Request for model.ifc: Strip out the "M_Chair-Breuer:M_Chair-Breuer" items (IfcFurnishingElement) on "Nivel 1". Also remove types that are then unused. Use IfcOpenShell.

First a look at what the model holds.

```python
import ifcopenshell
import ifcopenshell.util.element

model = ifcopenshell.open("model.ifc")
print(model.schema)
storey = next(s for s in model.by_type("IfcBuildingStorey") if s.Name == "Nivel 1")
furniture = [e for e in ifcopenshell.util.element.get_decomposition(storey) if e.is_a("IfcFurnishingElement")]
seen = {}
for e in furniture:
    element_type = ifcopenshell.util.element.get_type(e)
    name = element_type.Name if element_type not in (None, e) else None
    seen[name] = seen.get(name, 0) + 1
for name, count in sorted(seen.items(), key=str):
    print(count, "x", name)
```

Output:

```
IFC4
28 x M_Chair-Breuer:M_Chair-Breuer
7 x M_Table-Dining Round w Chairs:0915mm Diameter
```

```python
import ifcopenshell
import ifcopenshell.api.root
import ifcopenshell.util.element

model = ifcopenshell.open("model.ifc")

storey = next(s for s in model.by_type("IfcBuildingStorey") if s.Name == "Nivel 1")
furniture = [e for e in ifcopenshell.util.element.get_decomposition(storey) if e.is_a("IfcFurnishingElement")]
targets = [e for e in furniture if (t := ifcopenshell.util.element.get_type(e)) not in (None, e) and t.Name == "M_Chair-Breuer:M_Chair-Breuer"]
types = {ifcopenshell.util.element.get_type(e) for e in targets} - {None, *targets}

for e in targets:
    ifcopenshell.api.root.remove_product(model, product=e)
print(len(targets), "removed")

unused = [t for t in types if not ifcopenshell.util.element.get_types(t)]
for t in unused:
    ifcopenshell.api.root.remove_product(model, product=t)
print(len(unused), "unused types removed")

model.write("model_updated.ifc")
```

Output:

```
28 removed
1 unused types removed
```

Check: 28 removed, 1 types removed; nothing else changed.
